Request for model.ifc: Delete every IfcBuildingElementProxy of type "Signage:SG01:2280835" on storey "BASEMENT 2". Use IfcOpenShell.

First a look at what the model holds.

```python
import ifcopenshell
import ifcopenshell.util.element

model = ifcopenshell.open("model.ifc")
print(model.schema)
storey = next(s for s in model.by_type("IfcBuildingStorey") if s.Name == "BASEMENT 2")
proxies = [e for e in ifcopenshell.util.element.get_decomposition(storey) if e.is_a("IfcBuildingElementProxy")]
seen = {}
for e in proxies:
    element_type = ifcopenshell.util.element.get_type(e)
    name = element_type.Name if element_type not in (None, e) else None
    seen[name] = seen.get(name, 0) + 1
for name, count in sorted(seen.items(), key=str):
    print(count, "x", name)
```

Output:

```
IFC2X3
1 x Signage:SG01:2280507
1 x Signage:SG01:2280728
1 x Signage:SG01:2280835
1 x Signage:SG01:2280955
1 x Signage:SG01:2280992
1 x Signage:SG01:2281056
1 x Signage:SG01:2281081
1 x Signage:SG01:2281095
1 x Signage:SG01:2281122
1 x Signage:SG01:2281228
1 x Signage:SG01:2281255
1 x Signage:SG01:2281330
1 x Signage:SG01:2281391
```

```python
import ifcopenshell
import ifcopenshell.api.root
import ifcopenshell.util.element

model = ifcopenshell.open("model.ifc")

storey = next(s for s in model.by_type("IfcBuildingStorey") if s.Name == "BASEMENT 2")
proxies = [e for e in ifcopenshell.util.element.get_decomposition(storey) if e.is_a("IfcBuildingElementProxy")]
targets = [e for e in proxies if (t := ifcopenshell.util.element.get_type(e)) not in (None, e) and t.Name == "Signage:SG01:2280835"]

for e in targets:
    ifcopenshell.api.root.remove_product(model, product=e)
print(len(targets), "removed")

model.write("model_rev.ifc")
```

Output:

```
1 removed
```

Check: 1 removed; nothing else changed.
